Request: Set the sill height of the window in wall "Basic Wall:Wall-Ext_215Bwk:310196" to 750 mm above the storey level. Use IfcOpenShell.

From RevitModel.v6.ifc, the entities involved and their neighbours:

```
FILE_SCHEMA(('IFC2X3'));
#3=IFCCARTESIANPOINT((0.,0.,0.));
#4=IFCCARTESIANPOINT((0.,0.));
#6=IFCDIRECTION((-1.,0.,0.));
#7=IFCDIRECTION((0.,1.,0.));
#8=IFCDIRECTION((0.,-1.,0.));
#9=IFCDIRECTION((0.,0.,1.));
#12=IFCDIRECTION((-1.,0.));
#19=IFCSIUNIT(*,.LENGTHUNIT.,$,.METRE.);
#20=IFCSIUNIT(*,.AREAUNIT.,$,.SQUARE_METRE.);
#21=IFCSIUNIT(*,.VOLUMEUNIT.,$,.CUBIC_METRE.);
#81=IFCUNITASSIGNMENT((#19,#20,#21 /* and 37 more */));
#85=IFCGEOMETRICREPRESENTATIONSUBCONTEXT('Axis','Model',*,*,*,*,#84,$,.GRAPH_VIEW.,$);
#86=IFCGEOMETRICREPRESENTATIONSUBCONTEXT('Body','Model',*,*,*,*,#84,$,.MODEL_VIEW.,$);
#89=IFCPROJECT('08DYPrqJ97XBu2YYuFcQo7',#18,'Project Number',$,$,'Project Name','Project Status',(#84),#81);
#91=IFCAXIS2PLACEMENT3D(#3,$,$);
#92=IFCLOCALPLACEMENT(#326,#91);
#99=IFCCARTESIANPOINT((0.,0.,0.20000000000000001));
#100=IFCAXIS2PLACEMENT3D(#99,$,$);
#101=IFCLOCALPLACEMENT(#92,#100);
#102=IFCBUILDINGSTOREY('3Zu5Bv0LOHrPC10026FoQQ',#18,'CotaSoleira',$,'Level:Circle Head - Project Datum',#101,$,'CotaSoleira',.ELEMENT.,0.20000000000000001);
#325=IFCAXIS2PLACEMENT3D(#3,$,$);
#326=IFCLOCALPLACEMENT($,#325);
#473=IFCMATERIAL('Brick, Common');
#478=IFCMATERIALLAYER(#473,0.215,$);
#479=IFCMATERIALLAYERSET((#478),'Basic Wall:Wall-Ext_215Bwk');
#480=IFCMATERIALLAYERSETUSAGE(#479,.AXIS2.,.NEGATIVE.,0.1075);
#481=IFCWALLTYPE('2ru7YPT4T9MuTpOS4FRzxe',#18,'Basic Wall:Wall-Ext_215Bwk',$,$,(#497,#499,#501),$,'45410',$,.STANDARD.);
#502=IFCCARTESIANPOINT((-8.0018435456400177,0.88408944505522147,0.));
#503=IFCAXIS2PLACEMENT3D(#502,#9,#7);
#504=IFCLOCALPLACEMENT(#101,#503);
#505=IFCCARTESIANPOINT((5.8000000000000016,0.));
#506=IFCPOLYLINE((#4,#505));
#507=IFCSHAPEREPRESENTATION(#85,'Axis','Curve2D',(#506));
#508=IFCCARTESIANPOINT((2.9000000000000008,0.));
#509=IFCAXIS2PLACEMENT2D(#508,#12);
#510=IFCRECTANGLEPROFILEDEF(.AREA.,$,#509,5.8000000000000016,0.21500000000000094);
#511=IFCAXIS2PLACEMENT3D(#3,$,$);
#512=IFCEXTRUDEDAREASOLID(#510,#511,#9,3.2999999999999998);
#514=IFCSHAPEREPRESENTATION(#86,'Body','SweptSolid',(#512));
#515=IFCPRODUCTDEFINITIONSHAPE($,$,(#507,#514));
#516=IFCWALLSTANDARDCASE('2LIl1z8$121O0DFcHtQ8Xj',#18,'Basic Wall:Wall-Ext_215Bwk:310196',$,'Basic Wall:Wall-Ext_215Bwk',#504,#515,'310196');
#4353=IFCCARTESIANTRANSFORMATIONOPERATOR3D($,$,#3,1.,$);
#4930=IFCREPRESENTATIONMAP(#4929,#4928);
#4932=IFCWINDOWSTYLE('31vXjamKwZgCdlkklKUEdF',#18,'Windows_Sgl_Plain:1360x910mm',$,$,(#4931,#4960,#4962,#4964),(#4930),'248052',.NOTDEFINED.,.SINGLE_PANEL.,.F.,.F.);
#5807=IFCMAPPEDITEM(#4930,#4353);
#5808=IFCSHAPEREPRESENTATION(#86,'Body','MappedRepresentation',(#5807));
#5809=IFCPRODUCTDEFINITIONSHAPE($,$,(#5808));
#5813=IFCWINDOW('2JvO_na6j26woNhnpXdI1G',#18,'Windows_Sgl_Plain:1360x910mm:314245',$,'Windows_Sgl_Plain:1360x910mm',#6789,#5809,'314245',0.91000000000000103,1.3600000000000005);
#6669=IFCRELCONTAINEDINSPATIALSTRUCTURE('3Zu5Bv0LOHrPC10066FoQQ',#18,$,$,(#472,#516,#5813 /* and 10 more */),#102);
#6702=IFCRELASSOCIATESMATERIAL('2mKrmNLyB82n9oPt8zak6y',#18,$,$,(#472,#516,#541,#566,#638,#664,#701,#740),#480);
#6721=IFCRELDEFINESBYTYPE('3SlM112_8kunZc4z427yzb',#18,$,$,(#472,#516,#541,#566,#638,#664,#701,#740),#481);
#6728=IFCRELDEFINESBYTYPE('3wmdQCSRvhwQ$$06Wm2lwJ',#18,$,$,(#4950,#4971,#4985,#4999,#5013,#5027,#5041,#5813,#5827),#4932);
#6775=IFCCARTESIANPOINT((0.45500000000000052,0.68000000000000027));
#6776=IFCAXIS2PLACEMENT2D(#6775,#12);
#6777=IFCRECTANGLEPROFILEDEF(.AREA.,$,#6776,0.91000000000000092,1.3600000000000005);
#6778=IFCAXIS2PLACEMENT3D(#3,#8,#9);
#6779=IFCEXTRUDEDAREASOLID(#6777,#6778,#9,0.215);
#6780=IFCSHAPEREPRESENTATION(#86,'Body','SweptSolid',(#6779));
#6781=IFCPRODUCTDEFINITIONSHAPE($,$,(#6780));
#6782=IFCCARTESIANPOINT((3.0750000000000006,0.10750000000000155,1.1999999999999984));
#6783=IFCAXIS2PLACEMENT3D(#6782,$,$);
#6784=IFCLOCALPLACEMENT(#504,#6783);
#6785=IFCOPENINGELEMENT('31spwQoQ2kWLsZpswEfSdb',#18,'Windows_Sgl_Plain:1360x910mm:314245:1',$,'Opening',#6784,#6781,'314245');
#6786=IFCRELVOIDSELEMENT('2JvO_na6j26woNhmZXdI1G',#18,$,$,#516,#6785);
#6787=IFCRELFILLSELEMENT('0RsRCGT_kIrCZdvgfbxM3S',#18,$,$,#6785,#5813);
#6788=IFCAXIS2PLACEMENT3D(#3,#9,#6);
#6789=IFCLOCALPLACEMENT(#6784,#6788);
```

```python
import numpy as np
import ifcopenshell
import ifcopenshell.api.geometry
import ifcopenshell.geom
import ifcopenshell.util.element
import ifcopenshell.util.placement
import ifcopenshell.util.shape
import ifcopenshell.util.unit

model = ifcopenshell.open("RevitModel.v6.ifc")
unit_scale = ifcopenshell.util.unit.calculate_unit_scale(model)

window = model.by_guid("2JvO_na6j26woNhnpXdI1G")
opening = window.FillsVoids[0].RelatingOpeningElement
storey = ifcopenshell.util.element.get_container(window, ifc_class="IfcBuildingStorey")
level = ifcopenshell.util.placement.get_local_placement(storey.ObjectPlacement)[2, 3]

# The opening's origin need not be at the sill, so measure its lowest point.
shape = ifcopenshell.geom.create_shape(ifcopenshell.geom.settings(), opening)
bottom = ifcopenshell.util.shape.get_shape_bottom_elevation(shape, shape.geometry) / unit_scale
dz = level + 0.75 / unit_scale - bottom

shift = np.array([0.0, 0.0, dz])
# The window is placed relative to its opening, so it follows when the opening moves.
matrix = ifcopenshell.util.placement.get_local_placement(opening.ObjectPlacement)
matrix[:3, 3] += shift
ifcopenshell.api.geometry.edit_object_placement(
    model, product=opening, matrix=matrix, is_si=False, should_transform_children=True
)

print(f"moved by {dz * unit_scale:+.3f} m")

model.write("RevitModel.v6_updated.ifc")
```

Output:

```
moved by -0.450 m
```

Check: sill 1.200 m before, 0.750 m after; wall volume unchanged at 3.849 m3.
